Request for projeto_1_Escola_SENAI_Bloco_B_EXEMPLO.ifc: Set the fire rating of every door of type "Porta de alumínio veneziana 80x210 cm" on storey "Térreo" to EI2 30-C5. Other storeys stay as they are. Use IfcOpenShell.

First a look at what the model holds.

```python
import ifcopenshell
import ifcopenshell.util.element

model = ifcopenshell.open("projeto_1_Escola_SENAI_Bloco_B_EXEMPLO.ifc")
print(model.schema)
storey = next(s for s in model.by_type("IfcBuildingStorey") if s.Name == "Térreo")
doors = [e for e in ifcopenshell.util.element.get_decomposition(storey) if e.is_a("IfcDoor")]
seen = {}
for e in doors:
    element_type = ifcopenshell.util.element.get_type(e)
    key = (element_type.Name if element_type != e and element_type else None, ifcopenshell.util.element.get_pset(e, "Pset_DoorCommon", "FireRating"))
    seen[key] = seen.get(key, 0) + 1
for (name, value), count in sorted(seen.items(), key=str):
    print(count, "x", name, "|", value)
```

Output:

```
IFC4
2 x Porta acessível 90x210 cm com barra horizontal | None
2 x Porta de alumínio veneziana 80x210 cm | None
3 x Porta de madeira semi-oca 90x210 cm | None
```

```python
import ifcopenshell
import ifcopenshell.api.pset
import ifcopenshell.util.element

model = ifcopenshell.open("projeto_1_Escola_SENAI_Bloco_B_EXEMPLO.ifc")

storey = next(s for s in model.by_type("IfcBuildingStorey") if s.Name == "Térreo")
doors = [e for e in ifcopenshell.util.element.get_decomposition(storey) if e.is_a("IfcDoor")]

count = 0
for e in doors:
    element_type = ifcopenshell.util.element.get_type(e)
    if element_type in (None, e) or element_type.Name != "Porta de alumínio veneziana 80x210 cm":
        continue
    # add_pset returns the element's existing set when there is one.
    pset = ifcopenshell.api.pset.add_pset(model, product=e, name="Pset_DoorCommon")
    ifcopenshell.api.pset.edit_pset(model, pset=pset, properties={"FireRating": "EI2 30-C5"})
    count += 1

print(count, "doors updated")

model.write("projeto_1_Escola_SENAI_Bloco_B_EXEMPLO_rev.ifc")
```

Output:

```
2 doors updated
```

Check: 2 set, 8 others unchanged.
